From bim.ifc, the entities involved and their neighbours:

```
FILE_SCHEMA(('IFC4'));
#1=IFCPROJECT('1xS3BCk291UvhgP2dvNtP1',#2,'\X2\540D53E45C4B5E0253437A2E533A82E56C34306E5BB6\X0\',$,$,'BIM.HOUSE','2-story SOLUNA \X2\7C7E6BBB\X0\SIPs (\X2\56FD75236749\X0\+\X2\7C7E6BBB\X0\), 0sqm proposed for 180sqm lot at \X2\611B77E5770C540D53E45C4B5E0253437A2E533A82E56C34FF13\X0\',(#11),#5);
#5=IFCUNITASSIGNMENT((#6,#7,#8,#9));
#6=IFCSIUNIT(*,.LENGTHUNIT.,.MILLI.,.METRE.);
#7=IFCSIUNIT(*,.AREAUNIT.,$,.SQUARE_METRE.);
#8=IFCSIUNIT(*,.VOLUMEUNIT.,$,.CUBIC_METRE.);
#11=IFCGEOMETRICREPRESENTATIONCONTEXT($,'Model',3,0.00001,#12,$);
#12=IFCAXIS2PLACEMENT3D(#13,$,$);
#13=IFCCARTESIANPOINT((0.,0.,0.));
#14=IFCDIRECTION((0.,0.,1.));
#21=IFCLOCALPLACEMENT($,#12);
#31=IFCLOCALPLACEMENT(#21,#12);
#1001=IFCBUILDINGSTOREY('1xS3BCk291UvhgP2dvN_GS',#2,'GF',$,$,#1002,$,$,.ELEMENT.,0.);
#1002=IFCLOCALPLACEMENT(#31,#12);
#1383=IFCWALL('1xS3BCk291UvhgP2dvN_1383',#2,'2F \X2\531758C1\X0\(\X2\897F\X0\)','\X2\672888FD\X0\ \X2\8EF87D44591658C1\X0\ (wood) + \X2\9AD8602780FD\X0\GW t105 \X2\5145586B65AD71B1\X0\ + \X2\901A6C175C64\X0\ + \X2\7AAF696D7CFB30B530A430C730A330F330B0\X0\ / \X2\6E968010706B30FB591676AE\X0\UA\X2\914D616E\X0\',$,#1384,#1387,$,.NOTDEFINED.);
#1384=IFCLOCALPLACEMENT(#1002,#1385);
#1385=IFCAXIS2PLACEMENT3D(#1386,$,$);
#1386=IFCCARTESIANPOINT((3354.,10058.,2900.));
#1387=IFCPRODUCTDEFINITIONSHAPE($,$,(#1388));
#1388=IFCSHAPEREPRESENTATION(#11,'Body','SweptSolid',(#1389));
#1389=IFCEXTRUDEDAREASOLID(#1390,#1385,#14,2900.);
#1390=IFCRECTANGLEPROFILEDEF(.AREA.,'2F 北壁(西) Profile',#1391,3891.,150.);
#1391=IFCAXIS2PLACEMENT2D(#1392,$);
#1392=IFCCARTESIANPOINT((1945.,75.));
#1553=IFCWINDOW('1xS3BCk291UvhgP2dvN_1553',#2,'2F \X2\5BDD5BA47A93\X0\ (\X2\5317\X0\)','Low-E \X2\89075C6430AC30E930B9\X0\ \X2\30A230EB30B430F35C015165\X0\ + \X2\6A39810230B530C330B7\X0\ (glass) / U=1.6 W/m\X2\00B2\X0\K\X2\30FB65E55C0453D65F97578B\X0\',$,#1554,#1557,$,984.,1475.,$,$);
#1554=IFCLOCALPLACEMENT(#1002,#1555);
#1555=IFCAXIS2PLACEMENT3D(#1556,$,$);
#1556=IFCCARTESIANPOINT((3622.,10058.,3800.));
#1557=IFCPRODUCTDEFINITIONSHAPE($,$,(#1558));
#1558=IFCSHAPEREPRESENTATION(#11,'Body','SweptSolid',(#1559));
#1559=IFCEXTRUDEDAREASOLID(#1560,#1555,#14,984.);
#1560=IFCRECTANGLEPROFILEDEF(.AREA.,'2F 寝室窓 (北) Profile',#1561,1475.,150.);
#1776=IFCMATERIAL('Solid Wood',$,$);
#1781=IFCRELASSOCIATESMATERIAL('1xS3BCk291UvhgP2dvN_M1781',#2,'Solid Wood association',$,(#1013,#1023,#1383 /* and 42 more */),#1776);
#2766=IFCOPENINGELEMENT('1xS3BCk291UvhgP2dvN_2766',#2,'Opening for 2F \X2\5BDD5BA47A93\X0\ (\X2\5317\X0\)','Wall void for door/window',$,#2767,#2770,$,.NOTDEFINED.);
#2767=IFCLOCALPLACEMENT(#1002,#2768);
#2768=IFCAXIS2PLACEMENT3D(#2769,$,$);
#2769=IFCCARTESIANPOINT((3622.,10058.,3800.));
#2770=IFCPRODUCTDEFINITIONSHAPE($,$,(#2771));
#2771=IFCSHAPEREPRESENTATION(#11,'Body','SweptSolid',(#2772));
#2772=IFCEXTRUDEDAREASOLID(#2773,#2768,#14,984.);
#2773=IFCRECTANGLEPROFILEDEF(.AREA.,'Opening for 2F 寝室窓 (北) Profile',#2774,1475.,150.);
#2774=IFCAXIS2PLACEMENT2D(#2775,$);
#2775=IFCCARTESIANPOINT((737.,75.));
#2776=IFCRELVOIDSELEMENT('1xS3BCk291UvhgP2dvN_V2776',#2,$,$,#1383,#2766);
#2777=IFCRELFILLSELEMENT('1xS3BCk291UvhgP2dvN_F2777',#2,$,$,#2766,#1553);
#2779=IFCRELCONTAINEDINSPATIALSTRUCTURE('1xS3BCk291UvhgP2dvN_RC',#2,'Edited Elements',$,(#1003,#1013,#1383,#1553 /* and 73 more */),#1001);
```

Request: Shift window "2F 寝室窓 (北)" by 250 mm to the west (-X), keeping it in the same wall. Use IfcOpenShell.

```python
import ifcopenshell
import ifcopenshell.api.geometry
import ifcopenshell.util.placement
import ifcopenshell.util.unit

model = ifcopenshell.open("bim.ifc")
unit_scale = ifcopenshell.util.unit.calculate_unit_scale(model)

window = model.by_guid("1xS3BCk291UvhgP2dvN_1553")
opening = window.FillsVoids[0].RelatingOpeningElement
wall = opening.VoidsElements[0].RelatingBuildingElement

wall_matrix = ifcopenshell.util.placement.get_local_placement(wall.ObjectPlacement)
shift = wall_matrix[:3, 0] * -0.25 / unit_scale
before = ifcopenshell.util.placement.get_local_placement(window.ObjectPlacement)[:3, 3].copy()

# The window is not placed relative to its opening, so move both.
for product in (opening, window):
    matrix = ifcopenshell.util.placement.get_local_placement(product.ObjectPlacement)
    matrix[:3, 3] += shift
    ifcopenshell.api.geometry.edit_object_placement(model, product=product, matrix=matrix, is_si=False)

after = ifcopenshell.util.placement.get_local_placement(window.ObjectPlacement)[:3, 3]
print("window moved by", (after - before).round(3) + 0.0)

model.write("bim_rev.ifc")
```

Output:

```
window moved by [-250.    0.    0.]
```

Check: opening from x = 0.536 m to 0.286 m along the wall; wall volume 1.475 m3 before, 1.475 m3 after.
